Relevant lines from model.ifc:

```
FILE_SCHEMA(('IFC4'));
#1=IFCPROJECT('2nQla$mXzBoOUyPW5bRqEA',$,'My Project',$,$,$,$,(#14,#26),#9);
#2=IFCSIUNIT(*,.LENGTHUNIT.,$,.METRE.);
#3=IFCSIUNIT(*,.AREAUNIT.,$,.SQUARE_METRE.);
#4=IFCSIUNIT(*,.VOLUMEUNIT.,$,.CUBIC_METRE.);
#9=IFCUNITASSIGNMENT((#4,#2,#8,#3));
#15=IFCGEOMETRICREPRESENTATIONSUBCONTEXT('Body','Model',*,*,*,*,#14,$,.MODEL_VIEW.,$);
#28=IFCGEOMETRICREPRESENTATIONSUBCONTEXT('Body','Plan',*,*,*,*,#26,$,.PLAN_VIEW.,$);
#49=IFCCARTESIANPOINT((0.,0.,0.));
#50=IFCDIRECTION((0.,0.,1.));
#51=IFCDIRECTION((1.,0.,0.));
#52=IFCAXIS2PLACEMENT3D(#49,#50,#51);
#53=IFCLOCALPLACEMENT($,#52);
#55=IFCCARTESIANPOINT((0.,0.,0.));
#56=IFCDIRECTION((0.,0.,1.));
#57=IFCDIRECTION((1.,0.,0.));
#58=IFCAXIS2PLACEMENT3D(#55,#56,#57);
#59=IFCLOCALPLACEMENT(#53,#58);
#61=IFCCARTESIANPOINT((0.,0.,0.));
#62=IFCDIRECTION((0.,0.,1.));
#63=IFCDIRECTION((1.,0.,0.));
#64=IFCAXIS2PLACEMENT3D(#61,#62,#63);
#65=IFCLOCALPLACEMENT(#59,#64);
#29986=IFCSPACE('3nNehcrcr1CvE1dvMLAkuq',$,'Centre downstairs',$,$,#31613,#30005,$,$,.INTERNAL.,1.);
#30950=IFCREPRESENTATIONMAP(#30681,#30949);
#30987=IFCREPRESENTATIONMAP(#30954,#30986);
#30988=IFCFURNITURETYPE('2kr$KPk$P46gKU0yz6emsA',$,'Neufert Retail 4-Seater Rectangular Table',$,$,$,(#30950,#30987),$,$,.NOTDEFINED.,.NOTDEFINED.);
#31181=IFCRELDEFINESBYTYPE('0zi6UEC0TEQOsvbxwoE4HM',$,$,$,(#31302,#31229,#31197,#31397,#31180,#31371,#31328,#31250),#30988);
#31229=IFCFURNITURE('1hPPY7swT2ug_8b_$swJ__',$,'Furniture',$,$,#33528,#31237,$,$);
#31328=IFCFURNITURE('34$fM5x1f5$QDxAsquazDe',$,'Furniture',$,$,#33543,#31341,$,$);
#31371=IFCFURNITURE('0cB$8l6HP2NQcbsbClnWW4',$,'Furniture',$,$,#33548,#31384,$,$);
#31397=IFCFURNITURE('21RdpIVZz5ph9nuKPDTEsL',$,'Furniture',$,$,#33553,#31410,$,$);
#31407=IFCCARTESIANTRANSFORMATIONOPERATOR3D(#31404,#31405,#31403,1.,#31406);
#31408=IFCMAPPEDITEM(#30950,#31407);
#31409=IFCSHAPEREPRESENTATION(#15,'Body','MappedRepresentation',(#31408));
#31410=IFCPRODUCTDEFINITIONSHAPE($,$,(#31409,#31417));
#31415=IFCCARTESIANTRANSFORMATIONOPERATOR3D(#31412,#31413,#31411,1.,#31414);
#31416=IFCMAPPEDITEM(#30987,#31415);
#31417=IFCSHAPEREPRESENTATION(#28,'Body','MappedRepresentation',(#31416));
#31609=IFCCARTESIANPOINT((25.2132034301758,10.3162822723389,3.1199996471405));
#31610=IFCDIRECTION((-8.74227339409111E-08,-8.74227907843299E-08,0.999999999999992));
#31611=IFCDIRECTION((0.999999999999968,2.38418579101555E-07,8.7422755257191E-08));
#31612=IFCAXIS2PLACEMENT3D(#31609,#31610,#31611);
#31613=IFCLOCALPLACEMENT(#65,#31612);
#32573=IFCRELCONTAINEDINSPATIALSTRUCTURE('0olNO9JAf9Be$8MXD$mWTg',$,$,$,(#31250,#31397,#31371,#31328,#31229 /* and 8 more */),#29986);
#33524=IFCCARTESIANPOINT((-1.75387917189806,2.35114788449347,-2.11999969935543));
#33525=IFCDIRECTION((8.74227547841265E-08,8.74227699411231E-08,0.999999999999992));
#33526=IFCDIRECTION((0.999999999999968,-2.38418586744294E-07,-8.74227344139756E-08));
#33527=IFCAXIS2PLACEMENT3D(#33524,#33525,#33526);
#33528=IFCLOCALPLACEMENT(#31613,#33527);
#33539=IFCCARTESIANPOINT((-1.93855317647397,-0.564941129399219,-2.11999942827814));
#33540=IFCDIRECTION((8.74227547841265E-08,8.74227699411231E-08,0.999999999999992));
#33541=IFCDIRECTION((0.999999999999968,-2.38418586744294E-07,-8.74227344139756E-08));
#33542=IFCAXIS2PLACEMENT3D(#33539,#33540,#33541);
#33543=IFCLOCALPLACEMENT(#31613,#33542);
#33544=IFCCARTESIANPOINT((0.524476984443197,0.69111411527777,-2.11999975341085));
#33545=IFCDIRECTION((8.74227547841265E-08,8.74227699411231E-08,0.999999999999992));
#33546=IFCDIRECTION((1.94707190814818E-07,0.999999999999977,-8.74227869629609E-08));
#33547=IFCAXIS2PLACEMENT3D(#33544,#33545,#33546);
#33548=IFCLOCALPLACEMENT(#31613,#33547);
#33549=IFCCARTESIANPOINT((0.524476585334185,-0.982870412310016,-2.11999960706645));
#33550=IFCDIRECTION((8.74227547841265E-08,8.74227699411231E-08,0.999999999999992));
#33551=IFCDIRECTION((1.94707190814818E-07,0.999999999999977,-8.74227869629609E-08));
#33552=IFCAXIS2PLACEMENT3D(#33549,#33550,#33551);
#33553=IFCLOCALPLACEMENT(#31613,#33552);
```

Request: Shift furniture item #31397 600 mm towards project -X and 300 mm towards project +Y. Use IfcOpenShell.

```python
import ifcopenshell
import ifcopenshell.api.geometry
import ifcopenshell.util.placement
import ifcopenshell.util.unit

model = ifcopenshell.open("model.ifc")
unit_scale = ifcopenshell.util.unit.calculate_unit_scale(model)

item = model.by_id(31397)
matrix = ifcopenshell.util.placement.get_local_placement(item.ObjectPlacement)
matrix[0, 3] -= 0.6 / unit_scale
matrix[1, 3] += 0.3 / unit_scale
ifcopenshell.api.geometry.edit_object_placement(model, product=item, matrix=matrix, is_si=False)

print(ifcopenshell.util.placement.get_local_placement(item.ObjectPlacement).round(3) + 0.0)

model.write("model_edited.ifc")
```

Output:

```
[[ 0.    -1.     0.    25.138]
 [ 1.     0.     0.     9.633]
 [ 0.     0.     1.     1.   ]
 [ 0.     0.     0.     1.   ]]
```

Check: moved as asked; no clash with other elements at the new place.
